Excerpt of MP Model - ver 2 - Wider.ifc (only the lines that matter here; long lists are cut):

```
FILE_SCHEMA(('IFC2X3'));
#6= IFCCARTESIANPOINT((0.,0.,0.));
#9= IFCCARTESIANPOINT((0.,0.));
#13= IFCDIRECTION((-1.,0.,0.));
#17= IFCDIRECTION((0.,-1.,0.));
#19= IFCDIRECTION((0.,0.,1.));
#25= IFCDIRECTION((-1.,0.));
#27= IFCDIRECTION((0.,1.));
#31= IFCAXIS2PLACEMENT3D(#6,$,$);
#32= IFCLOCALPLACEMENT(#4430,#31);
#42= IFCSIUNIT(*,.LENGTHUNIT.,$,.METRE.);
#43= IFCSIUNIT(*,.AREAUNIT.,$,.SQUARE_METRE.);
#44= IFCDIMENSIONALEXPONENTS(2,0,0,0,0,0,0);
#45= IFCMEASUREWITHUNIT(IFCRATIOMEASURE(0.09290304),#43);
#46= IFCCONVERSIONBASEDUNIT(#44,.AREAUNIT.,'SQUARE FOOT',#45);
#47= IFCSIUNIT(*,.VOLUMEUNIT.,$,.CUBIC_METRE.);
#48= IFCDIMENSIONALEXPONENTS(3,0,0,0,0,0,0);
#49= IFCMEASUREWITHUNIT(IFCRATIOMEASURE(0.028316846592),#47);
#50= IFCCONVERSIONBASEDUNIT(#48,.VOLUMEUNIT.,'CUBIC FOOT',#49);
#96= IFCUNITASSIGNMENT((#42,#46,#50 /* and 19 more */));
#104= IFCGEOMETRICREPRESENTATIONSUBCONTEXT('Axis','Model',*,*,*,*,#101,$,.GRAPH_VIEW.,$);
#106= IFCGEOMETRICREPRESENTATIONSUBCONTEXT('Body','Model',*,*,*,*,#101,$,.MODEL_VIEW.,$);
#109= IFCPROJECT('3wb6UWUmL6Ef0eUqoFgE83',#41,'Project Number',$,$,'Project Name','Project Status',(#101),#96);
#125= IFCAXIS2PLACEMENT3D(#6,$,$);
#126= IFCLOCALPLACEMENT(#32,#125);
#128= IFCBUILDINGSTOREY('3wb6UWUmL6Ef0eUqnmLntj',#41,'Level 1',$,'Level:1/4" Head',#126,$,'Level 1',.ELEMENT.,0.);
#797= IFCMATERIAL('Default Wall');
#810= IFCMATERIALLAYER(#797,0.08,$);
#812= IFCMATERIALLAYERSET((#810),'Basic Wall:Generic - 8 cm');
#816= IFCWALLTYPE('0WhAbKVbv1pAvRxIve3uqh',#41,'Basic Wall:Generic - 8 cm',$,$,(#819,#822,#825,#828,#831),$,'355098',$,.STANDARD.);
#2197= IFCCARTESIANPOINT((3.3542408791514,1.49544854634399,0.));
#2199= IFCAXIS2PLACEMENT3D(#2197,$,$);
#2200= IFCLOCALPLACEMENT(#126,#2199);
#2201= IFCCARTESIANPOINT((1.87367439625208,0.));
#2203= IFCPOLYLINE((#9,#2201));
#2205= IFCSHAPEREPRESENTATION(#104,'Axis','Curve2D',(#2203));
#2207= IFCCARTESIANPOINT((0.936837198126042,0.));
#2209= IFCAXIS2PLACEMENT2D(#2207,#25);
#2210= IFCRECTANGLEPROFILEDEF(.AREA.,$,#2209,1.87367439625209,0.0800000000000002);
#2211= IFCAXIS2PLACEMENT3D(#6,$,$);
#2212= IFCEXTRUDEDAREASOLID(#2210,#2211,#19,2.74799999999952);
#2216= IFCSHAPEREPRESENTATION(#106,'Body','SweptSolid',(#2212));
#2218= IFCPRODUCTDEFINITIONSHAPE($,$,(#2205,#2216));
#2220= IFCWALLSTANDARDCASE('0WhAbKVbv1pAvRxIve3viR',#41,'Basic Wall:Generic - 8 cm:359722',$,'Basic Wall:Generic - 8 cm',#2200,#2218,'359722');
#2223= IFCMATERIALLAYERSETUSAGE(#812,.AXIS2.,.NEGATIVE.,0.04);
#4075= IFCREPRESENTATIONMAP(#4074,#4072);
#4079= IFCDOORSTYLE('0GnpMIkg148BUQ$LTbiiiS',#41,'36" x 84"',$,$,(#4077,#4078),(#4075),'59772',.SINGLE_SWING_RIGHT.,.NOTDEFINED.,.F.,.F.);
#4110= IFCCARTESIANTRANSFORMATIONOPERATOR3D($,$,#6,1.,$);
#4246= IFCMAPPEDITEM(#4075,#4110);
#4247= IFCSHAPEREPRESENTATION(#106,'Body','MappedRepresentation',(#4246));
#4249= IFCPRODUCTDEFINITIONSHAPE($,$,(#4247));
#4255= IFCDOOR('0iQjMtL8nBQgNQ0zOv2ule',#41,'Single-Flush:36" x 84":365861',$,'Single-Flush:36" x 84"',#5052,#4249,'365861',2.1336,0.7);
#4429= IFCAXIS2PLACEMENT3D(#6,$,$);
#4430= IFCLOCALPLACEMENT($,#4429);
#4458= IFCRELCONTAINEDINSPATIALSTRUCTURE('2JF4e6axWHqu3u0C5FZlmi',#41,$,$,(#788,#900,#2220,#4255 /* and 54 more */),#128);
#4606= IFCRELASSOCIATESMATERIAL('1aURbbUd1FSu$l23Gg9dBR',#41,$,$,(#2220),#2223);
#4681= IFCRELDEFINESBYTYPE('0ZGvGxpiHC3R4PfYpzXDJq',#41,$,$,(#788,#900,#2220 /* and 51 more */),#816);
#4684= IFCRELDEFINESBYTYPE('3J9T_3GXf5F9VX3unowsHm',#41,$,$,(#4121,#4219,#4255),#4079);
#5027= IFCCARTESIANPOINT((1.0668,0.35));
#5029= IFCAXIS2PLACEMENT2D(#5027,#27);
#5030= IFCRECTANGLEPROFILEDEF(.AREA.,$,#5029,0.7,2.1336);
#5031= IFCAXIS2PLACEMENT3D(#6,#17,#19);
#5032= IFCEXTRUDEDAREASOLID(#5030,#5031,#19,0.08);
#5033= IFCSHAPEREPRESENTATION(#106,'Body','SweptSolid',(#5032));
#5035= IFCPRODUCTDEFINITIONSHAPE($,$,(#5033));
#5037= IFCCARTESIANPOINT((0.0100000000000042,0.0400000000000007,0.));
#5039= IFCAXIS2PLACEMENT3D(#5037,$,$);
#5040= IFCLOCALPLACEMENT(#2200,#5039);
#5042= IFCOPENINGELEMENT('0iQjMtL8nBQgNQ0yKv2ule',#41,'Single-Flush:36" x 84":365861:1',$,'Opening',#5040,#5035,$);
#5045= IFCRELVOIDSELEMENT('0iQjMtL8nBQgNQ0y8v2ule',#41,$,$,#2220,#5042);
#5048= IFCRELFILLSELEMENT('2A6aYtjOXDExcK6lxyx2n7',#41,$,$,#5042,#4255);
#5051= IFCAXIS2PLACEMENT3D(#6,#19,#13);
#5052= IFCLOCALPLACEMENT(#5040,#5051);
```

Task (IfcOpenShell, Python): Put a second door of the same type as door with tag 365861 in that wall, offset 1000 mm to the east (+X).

```python
import ifcopenshell
import ifcopenshell.api.feature
import ifcopenshell.api.geometry
import ifcopenshell.api.root
import ifcopenshell.geom
import ifcopenshell.util.element
import ifcopenshell.util.placement
import ifcopenshell.util.shape
import ifcopenshell.util.unit

model = ifcopenshell.open("MP Model - ver 2 - Wider.ifc")
unit_scale = ifcopenshell.util.unit.calculate_unit_scale(model)
settings = ifcopenshell.geom.settings()


def volume(element):
    """Net volume in cubic metres, openings subtracted."""
    shape = ifcopenshell.geom.create_shape(settings, element)
    return ifcopenshell.util.shape.get_volume(shape.geometry)


def reuse_history(source, copy):
    """copy_class also copies each property set's owner history, people and application; keep the originals."""
    for rel in copy.IsDefinedBy:
        if rel.is_a("IfcRelDefinesByProperties") and (history := rel.RelatingPropertyDefinition.OwnerHistory):
            rel.RelatingPropertyDefinition.OwnerHistory = source.OwnerHistory
            ifcopenshell.util.element.remove_deep2(model, history)


door = model.by_guid("0iQjMtL8nBQgNQ0zOv2ule")
opening = door.FillsVoids[0].RelatingOpeningElement
wall = opening.VoidsElements[0].RelatingBuildingElement
before = volume(wall)
shift = ifcopenshell.util.placement.get_local_placement(wall.ObjectPlacement)[:3, 0] * 1 / unit_scale

# copy_class copies the void relationship, type, container and properties, but no geometry.
new_opening = ifcopenshell.api.root.copy_class(model, product=opening)
new_opening.Representation = ifcopenshell.util.element.copy_deep(
    model, opening.Representation, exclude=["IfcGeometricRepresentationContext", "IfcRepresentationMap"]
)
new_opening.Name = 'Single-Flush:36" x 84"'
new_door = ifcopenshell.api.root.copy_class(model, product=door)
new_door.Representation = ifcopenshell.util.element.copy_deep(
    model, door.Representation, exclude=["IfcGeometricRepresentationContext", "IfcRepresentationMap"]
)
new_door.Name = 'Single-Flush:36" x 84"'
new_door.Tag = None
reuse_history(door, new_door)
fills = ifcopenshell.api.feature.add_filling(model, opening=new_opening, element=new_door)
fills.OwnerHistory = new_door.OwnerHistory  # required in IFC2X3

for old, new in ((opening, new_opening), (door, new_door)):
    matrix = ifcopenshell.util.placement.get_local_placement(old.ObjectPlacement)
    matrix[:3, 3] += shift
    ifcopenshell.api.geometry.edit_object_placement(model, product=new, matrix=matrix, is_si=False)

after = volume(wall)

print(f"wall volume {before:.3f} -> {after:.3f} m3")

model.write("MP Model - ver 2 - Wider_edited.ifc")
```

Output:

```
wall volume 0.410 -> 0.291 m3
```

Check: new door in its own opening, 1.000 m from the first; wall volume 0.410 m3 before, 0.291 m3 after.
